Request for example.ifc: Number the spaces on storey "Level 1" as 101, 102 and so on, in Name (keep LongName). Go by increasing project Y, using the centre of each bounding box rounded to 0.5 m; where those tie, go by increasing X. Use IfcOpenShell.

First a look at what the model holds.

```python
import ifcopenshell
import ifcopenshell.util.element
import ifcopenshell.util.placement

model = ifcopenshell.open("example.ifc")
print(model.schema)
storey = next(s for s in model.by_type("IfcBuildingStorey") if s.Name == "Level 1")
spaces = [e for e in ifcopenshell.util.element.get_decomposition(storey) if e.is_a("IfcSpace")]
for e in sorted(spaces, key=lambda e: e.id()):
    origin = ifcopenshell.util.placement.get_local_placement(e.ObjectPlacement)[:3, 3]
    print(e.id(), e.Name, e.LongName, origin.round(2) + 0.0, sep=" | ")
```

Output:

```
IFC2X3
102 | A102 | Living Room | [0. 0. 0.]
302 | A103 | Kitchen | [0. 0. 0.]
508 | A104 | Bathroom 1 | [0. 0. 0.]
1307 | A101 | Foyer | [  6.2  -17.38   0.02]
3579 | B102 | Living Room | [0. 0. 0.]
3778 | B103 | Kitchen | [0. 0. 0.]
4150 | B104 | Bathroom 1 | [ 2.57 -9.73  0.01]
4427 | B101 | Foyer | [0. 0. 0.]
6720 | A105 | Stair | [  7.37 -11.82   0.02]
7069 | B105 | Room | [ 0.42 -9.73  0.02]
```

```python
import ifcopenshell
import ifcopenshell.geom
import ifcopenshell.util.element
import ifcopenshell.util.shape

model = ifcopenshell.open("example.ifc")
settings = ifcopenshell.geom.settings()
settings.set("use-world-coords", True)


def centre(element):
    shape = ifcopenshell.geom.create_shape(settings, element)
    return ifcopenshell.util.shape.get_bbox_centroid(shape.geometry)


storey = next(s for s in model.by_type("IfcBuildingStorey") if s.Name == "Level 1")
spaces = [e for e in ifcopenshell.util.element.get_decomposition(storey) if e.is_a("IfcSpace")]

# Insertion points can sit at a corner or the storey origin, so sort by the geometry (in metres).
centres = {e: centre(e) for e in spaces}
spaces.sort(key=lambda e: (round(centres[e][1] / 0.5), centres[e][0]))

for i, e in enumerate(spaces, start=1):
    number = f"1{i:02d}"
    e.Name = number
    print(e.id(), number)

model.write("example_edited.ifc")
```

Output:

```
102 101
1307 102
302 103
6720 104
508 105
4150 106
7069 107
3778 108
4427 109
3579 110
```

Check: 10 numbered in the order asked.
